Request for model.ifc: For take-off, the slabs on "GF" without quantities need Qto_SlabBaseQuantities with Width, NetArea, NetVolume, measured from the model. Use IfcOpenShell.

First a look at what the model holds.

```python
import ifcopenshell
import ifcopenshell.util.element
import ifcopenshell.util.unit

model = ifcopenshell.open("model.ifc")
print(model.schema)
for unit_type in ("LENGTHUNIT", "AREAUNIT", "VOLUMEUNIT"):
    print(unit_type, ifcopenshell.util.unit.calculate_unit_scale(model, unit_type))
storey = next(s for s in model.by_type("IfcBuildingStorey") if s.Name == "GF")
slabs = [e for e in ifcopenshell.util.element.get_decomposition(storey) if e.is_a("IfcSlab")]
for e in sorted(slabs, key=lambda e: e.id()):
    print(e.id(), e.is_a(), e.Name, list(ifcopenshell.util.element.get_psets(e, qtos_only=True)), sep=" | ")
```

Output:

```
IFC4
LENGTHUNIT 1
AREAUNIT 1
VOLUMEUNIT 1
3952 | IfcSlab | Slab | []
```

```python
import ifcopenshell
import ifcopenshell.api.pset
import ifcopenshell.geom
import ifcopenshell.util.element
import ifcopenshell.util.shape
import ifcopenshell.util.unit

model = ifcopenshell.open("model.ifc")
unit_scale = ifcopenshell.util.unit.calculate_unit_scale(model)
area_scale = ifcopenshell.util.unit.calculate_unit_scale(model, "AREAUNIT")
volume_scale = ifcopenshell.util.unit.calculate_unit_scale(model, "VOLUMEUNIT")
settings = ifcopenshell.geom.settings()

storey = next(s for s in model.by_type("IfcBuildingStorey") if s.Name == "GF")
slabs = [e for e in ifcopenshell.util.element.get_decomposition(storey) if e.is_a("IfcSlab")]

for e in sorted(slabs, key=lambda e: e.id()):
    if ifcopenshell.util.element.get_psets(e, qtos_only=True, should_inherit=False):
        continue
    # Geometry comes back in metres, in the element's own axes.
    shape = ifcopenshell.geom.create_shape(settings, e)
    values = {
        "Width": ifcopenshell.util.shape.get_z(shape.geometry) / unit_scale,
        "NetArea": ifcopenshell.util.shape.get_footprint_area(shape.geometry) / area_scale,
        "NetVolume": ifcopenshell.util.shape.get_volume(shape.geometry) / volume_scale,
    }
    qto = ifcopenshell.api.pset.add_qto(model, product=e, name="Qto_SlabBaseQuantities")
    ifcopenshell.api.pset.edit_qto(model, qto=qto, properties=values)
    print(e.id(), {k: round(v, 3) for k, v in values.items()})

model.write("model_v2.ifc")
```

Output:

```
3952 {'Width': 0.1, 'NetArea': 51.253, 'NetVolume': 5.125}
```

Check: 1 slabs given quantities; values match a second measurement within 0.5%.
